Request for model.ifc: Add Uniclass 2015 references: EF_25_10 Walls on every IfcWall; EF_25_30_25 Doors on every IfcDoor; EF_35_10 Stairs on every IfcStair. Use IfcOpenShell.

First a look at what the model holds.

```python
import ifcopenshell

model = ifcopenshell.open("model.ifc")
print(model.schema)
print("classifications:", [c.Name for c in model.by_type("IfcClassification")])
for ifc_class in ("IfcDoor", "IfcRoof", "IfcStair", "IfcWall", "IfcWindow"):
    print(ifc_class, len(model.by_type(ifc_class)))
```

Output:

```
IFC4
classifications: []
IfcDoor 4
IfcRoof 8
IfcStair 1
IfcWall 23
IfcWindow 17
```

```python
import ifcopenshell
import ifcopenshell.api.classification

model = ifcopenshell.open("model.ifc")

system = ifcopenshell.api.classification.add_classification(model, classification="Uniclass 2015")

codes = {
    "IfcWall": ("EF_25_10", "Walls"),
    "IfcDoor": ("EF_25_30_25", "Doors"),
    "IfcStair": ("EF_35_10", "Stairs"),
}
for ifc_class, (code, name) in codes.items():
    products = model.by_type(ifc_class)
    ifcopenshell.api.classification.add_reference(
        model, products=products, classification=system, identification=code, name=name
    )
    print(code, len(products))

model.write("model_rev.ifc")
```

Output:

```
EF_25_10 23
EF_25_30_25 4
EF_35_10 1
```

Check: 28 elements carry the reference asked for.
